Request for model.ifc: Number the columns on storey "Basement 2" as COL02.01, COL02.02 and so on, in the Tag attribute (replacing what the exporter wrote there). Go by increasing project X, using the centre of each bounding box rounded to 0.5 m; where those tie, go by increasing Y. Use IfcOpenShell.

First a look at what the model holds.

```python
import ifcopenshell
import ifcopenshell.util.element
import ifcopenshell.util.placement

model = ifcopenshell.open("model.ifc")
print(model.schema)
storey = next(s for s in model.by_type("IfcBuildingStorey") if s.Name == "Basement 2")
columns = [e for e in ifcopenshell.util.element.get_decomposition(storey) if e.is_a("IfcColumn")]
for e in sorted(columns, key=lambda e: e.id()):
    origin = ifcopenshell.util.placement.get_local_placement(e.ObjectPlacement)[:3, 3]
    print(e.id(), e.Tag, e.Name, origin.round(2) + 0.0, sep=" | ")
```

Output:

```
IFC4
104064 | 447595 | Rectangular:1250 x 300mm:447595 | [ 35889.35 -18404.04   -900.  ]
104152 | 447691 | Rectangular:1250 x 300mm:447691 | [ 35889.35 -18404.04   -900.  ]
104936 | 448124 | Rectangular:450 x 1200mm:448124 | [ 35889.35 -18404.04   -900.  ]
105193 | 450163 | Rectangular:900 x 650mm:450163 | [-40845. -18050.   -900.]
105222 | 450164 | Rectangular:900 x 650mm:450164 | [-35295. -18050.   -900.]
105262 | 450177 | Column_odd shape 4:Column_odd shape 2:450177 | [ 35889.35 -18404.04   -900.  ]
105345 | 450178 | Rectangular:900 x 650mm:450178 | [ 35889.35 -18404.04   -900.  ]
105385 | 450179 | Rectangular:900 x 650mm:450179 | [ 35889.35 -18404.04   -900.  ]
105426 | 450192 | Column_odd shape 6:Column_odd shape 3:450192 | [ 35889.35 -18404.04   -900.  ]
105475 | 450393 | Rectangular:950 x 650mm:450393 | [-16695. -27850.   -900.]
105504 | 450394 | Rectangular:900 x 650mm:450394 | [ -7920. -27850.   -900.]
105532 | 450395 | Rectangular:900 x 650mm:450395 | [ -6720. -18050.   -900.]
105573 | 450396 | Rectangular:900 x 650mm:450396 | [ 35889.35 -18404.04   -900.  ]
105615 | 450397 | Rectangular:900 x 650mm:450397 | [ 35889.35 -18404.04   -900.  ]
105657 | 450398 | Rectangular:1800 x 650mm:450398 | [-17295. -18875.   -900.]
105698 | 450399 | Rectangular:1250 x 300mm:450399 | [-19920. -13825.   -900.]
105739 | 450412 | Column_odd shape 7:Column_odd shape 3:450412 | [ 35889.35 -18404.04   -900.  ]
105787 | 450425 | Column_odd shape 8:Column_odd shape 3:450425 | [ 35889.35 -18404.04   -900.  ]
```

```python
import ifcopenshell
import ifcopenshell.geom
import ifcopenshell.util.element
import ifcopenshell.util.shape

model = ifcopenshell.open("model.ifc")
settings = ifcopenshell.geom.settings()
settings.set("use-world-coords", True)


def centre(element):
    shape = ifcopenshell.geom.create_shape(settings, element)
    return ifcopenshell.util.shape.get_bbox_centroid(shape.geometry)


storey = next(s for s in model.by_type("IfcBuildingStorey") if s.Name == "Basement 2")
columns = [e for e in ifcopenshell.util.element.get_decomposition(storey) if e.is_a("IfcColumn")]

# Insertion points can sit at a corner or the storey origin, so sort by the geometry (in metres).
centres = {e: centre(e) for e in columns}
columns.sort(key=lambda e: (round(centres[e][0] / 0.5), centres[e][1]))

for i, e in enumerate(columns, start=1):
    number = f"COL02.{i:02d}"
    e.Tag = number
    print(e.id(), number)

model.write("model_updated.ifc")
```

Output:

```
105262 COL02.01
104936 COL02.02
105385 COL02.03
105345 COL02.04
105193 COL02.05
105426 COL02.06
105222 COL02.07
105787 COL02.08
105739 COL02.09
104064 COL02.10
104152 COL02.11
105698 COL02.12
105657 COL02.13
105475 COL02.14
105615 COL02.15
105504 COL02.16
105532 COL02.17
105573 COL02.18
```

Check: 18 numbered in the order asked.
